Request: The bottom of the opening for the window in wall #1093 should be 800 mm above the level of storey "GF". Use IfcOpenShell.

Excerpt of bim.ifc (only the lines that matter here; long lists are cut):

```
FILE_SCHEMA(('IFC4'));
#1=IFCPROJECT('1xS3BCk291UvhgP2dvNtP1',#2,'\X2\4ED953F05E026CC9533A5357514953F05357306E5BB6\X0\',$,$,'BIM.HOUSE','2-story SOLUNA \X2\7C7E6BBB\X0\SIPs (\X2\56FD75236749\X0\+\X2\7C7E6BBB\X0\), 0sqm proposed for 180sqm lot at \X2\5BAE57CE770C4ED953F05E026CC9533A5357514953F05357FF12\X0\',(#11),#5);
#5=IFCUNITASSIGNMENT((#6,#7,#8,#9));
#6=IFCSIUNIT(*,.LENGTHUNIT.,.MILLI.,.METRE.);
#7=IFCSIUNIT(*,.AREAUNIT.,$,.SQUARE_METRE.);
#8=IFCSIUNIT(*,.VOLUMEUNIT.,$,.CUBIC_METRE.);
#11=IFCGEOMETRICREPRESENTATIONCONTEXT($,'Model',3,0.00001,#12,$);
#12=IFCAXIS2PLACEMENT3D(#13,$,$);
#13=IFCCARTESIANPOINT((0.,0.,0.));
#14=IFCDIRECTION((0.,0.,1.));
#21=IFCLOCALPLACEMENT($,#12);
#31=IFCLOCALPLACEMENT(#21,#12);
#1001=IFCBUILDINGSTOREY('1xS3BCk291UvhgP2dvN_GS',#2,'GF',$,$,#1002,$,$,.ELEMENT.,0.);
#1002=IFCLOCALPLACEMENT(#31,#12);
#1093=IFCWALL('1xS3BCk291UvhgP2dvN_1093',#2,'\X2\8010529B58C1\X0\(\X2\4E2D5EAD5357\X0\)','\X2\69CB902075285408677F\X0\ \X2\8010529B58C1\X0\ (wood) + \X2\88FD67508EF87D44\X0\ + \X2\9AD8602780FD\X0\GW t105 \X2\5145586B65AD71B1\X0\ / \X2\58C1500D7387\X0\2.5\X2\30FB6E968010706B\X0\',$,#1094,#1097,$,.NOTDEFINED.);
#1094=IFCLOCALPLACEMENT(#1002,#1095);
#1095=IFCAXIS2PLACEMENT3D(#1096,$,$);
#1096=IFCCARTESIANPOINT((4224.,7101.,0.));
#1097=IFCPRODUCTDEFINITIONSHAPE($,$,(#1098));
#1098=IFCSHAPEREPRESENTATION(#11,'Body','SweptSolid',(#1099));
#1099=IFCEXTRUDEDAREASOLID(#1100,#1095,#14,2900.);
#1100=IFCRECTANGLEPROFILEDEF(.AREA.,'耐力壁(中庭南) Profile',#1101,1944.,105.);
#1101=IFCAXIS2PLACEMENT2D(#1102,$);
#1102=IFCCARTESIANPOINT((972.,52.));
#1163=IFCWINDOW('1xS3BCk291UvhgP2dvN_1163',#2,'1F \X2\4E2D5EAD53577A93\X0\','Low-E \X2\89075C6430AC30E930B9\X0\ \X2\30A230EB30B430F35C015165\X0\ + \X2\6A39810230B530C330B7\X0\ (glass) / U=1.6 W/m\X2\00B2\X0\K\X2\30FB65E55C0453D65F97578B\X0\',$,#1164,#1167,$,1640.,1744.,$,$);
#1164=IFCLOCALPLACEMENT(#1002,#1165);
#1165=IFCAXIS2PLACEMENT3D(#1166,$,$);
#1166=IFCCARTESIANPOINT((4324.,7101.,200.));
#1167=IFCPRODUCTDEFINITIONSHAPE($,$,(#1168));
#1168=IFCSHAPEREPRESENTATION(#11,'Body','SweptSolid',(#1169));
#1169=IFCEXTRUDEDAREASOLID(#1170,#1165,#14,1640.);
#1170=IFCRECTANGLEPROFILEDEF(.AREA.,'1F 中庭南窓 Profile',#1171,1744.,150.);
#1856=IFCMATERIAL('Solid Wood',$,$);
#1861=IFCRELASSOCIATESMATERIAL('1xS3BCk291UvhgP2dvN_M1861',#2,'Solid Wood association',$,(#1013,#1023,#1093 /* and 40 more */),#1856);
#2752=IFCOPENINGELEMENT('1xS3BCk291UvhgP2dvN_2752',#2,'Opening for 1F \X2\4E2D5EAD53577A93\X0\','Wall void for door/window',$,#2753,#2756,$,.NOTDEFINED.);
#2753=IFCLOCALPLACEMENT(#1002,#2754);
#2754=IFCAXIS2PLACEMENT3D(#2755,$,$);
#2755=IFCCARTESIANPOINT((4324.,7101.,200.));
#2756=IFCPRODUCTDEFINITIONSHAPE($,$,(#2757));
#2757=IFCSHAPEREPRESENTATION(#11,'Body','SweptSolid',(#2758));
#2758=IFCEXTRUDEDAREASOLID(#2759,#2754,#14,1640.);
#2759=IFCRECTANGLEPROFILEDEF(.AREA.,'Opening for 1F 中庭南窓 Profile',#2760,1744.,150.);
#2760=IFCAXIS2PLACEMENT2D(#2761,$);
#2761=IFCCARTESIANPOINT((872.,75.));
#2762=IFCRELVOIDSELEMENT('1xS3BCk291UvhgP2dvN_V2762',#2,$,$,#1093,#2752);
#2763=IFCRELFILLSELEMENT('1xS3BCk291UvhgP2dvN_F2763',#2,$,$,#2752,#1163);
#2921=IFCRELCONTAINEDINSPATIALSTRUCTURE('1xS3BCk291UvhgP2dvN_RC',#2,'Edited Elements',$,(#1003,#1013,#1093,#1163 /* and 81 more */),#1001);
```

```python
import numpy as np
import ifcopenshell
import ifcopenshell.api.geometry
import ifcopenshell.geom
import ifcopenshell.util.element
import ifcopenshell.util.placement
import ifcopenshell.util.shape
import ifcopenshell.util.unit

model = ifcopenshell.open("bim.ifc")
unit_scale = ifcopenshell.util.unit.calculate_unit_scale(model)

window = model.by_guid("1xS3BCk291UvhgP2dvN_1163")
opening = window.FillsVoids[0].RelatingOpeningElement
storey = ifcopenshell.util.element.get_container(window, ifc_class="IfcBuildingStorey")
level = ifcopenshell.util.placement.get_local_placement(storey.ObjectPlacement)[2, 3]

# The opening's origin need not be at the sill, so measure its lowest point.
shape = ifcopenshell.geom.create_shape(ifcopenshell.geom.settings(), opening)
bottom = ifcopenshell.util.shape.get_shape_bottom_elevation(shape, shape.geometry) / unit_scale
dz = level + 0.8 / unit_scale - bottom

shift = np.array([0.0, 0.0, dz])
# The window is not placed relative to its opening, so move both.
for product in (opening, window):
    matrix = ifcopenshell.util.placement.get_local_placement(product.ObjectPlacement)
    matrix[:3, 3] += shift
    ifcopenshell.api.geometry.edit_object_placement(model, product=product, matrix=matrix, is_si=False)

print(f"moved by {dz * unit_scale:+.3f} m")

model.write("bim_updated.ifc")
```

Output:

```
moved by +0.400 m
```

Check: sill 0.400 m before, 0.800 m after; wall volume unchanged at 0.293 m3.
